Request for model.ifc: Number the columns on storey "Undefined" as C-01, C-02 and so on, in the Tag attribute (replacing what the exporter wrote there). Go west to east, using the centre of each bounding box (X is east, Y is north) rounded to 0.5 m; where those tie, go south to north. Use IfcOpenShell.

First a look at what the model holds.

```python
import ifcopenshell
import ifcopenshell.util.element
import ifcopenshell.util.placement

model = ifcopenshell.open("model.ifc")
print(model.schema)
storey = next(s for s in model.by_type("IfcBuildingStorey") if s.Name == "Undefined")
columns = [e for e in ifcopenshell.util.element.get_decomposition(storey) if e.is_a("IfcColumn")]
for e in sorted(columns, key=lambda e: e.id()):
    origin = ifcopenshell.util.placement.get_local_placement(e.ObjectPlacement)[:3, 3]
    print(e.id(), e.Tag, e.Name, origin.round(2) + 0.0, sep=" | ")
```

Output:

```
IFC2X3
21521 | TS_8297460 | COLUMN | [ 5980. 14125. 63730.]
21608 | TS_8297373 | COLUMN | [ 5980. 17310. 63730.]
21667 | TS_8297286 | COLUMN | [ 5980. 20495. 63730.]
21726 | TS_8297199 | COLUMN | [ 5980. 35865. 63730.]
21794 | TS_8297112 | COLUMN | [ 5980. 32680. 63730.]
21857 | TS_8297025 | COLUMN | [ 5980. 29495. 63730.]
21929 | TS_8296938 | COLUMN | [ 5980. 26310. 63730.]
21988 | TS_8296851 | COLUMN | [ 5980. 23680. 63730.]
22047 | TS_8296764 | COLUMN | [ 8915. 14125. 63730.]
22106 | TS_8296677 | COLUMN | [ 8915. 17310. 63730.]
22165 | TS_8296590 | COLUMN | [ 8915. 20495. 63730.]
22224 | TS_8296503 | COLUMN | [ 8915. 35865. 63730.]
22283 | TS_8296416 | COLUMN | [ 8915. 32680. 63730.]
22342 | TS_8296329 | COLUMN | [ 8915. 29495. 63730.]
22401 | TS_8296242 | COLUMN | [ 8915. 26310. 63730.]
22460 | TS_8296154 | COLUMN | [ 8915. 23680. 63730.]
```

```python
import ifcopenshell
import ifcopenshell.geom
import ifcopenshell.util.element
import ifcopenshell.util.shape

model = ifcopenshell.open("model.ifc")
settings = ifcopenshell.geom.settings()
settings.set("use-world-coords", True)


def centre(element):
    shape = ifcopenshell.geom.create_shape(settings, element)
    return ifcopenshell.util.shape.get_bbox_centroid(shape.geometry)


storey = next(s for s in model.by_type("IfcBuildingStorey") if s.Name == "Undefined")
columns = [e for e in ifcopenshell.util.element.get_decomposition(storey) if e.is_a("IfcColumn")]

# Insertion points can sit at a corner or the storey origin, so sort by the geometry (in metres).
centres = {e: centre(e) for e in columns}
columns.sort(key=lambda e: (round(centres[e][0] / 0.5), centres[e][1]))

for i, e in enumerate(columns, start=1):
    number = f"C-{i:02d}"
    e.Tag = number
    print(e.id(), number)

model.write("model-out.ifc")
```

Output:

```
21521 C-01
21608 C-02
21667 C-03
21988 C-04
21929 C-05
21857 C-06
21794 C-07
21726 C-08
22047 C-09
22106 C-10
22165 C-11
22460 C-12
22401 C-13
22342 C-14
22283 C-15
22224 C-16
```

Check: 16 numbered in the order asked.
